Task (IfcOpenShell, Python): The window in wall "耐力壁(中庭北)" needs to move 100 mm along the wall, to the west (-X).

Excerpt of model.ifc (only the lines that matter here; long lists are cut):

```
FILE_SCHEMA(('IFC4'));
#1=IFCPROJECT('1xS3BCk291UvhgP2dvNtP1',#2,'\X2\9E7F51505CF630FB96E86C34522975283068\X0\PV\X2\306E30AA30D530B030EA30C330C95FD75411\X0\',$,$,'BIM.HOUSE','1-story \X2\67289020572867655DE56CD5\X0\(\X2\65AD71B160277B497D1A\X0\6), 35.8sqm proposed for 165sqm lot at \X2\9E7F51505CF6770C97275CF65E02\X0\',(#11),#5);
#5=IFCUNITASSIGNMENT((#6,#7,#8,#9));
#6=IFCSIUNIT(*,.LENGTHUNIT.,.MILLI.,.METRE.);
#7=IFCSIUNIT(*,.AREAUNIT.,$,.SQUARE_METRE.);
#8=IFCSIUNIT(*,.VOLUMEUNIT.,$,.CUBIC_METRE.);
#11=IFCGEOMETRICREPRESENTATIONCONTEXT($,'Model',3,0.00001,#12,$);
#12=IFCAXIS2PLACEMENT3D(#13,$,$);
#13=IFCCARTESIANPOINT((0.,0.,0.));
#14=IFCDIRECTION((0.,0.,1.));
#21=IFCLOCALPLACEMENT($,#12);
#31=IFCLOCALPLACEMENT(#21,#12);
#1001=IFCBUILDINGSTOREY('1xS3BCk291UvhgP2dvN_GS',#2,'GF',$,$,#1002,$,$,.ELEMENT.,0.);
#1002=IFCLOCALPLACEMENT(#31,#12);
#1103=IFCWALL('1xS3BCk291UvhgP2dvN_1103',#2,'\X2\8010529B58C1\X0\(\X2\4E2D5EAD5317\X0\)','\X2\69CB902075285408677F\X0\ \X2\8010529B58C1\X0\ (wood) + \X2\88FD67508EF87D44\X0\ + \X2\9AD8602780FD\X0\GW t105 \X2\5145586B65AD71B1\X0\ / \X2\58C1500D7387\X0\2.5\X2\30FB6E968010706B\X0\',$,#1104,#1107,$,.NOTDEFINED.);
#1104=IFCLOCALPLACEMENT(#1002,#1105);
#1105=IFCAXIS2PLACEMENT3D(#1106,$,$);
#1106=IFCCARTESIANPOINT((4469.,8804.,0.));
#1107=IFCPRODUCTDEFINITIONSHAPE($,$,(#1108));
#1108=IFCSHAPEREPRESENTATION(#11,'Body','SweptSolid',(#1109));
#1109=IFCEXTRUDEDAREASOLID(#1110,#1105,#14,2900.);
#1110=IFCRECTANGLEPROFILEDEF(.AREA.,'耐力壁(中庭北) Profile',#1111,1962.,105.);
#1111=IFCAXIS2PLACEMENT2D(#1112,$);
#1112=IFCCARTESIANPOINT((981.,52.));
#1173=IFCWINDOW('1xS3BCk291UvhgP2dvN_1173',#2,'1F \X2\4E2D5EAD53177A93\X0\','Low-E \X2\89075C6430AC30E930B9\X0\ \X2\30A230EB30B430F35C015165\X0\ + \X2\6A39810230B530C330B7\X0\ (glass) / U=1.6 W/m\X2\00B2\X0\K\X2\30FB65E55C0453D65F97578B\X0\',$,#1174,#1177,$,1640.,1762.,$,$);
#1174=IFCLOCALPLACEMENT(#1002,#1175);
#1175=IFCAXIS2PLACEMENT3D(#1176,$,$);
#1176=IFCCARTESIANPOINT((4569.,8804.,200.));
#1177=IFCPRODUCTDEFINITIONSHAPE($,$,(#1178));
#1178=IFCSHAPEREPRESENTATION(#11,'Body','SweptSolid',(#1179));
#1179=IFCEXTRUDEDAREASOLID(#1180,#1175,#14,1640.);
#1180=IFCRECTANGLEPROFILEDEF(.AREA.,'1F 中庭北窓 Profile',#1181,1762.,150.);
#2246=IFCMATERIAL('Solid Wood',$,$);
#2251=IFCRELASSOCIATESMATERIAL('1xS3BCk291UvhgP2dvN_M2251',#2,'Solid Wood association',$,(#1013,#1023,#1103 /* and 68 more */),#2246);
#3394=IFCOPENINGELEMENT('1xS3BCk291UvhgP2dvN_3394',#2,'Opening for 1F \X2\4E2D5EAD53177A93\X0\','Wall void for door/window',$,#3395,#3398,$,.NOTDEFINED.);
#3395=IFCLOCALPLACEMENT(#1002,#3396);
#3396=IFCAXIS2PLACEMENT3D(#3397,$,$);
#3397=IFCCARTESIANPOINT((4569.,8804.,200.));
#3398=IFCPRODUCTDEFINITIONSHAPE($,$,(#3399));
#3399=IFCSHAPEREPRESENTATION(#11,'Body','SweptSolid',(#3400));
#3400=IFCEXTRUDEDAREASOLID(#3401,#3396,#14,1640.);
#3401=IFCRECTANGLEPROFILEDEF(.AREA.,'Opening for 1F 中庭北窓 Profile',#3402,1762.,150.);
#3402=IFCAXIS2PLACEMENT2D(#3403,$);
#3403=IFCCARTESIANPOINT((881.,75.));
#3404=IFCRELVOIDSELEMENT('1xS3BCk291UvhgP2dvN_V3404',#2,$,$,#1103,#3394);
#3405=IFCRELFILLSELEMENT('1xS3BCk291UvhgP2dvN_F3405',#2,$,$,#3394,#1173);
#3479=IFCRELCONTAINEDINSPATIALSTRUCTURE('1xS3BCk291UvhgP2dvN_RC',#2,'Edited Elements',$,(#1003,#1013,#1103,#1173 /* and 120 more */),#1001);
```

```python
import ifcopenshell
import ifcopenshell.api.geometry
import ifcopenshell.util.placement
import ifcopenshell.util.unit

model = ifcopenshell.open("model.ifc")
unit_scale = ifcopenshell.util.unit.calculate_unit_scale(model)

window = model.by_id(1173)
opening = window.FillsVoids[0].RelatingOpeningElement
wall = opening.VoidsElements[0].RelatingBuildingElement

wall_matrix = ifcopenshell.util.placement.get_local_placement(wall.ObjectPlacement)
shift = wall_matrix[:3, 0] * -0.1 / unit_scale
before = ifcopenshell.util.placement.get_local_placement(window.ObjectPlacement)[:3, 3].copy()

# The window is not placed relative to its opening, so move both.
for product in (opening, window):
    matrix = ifcopenshell.util.placement.get_local_placement(product.ObjectPlacement)
    matrix[:3, 3] += shift
    ifcopenshell.api.geometry.edit_object_placement(model, product=product, matrix=matrix, is_si=False)

after = ifcopenshell.util.placement.get_local_placement(window.ObjectPlacement)[:3, 3]
print("window moved by", (after - before).round(3) + 0.0)

model.write("model_rev.ifc")
```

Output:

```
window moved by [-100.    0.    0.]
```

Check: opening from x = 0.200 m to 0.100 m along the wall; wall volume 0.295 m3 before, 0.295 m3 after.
